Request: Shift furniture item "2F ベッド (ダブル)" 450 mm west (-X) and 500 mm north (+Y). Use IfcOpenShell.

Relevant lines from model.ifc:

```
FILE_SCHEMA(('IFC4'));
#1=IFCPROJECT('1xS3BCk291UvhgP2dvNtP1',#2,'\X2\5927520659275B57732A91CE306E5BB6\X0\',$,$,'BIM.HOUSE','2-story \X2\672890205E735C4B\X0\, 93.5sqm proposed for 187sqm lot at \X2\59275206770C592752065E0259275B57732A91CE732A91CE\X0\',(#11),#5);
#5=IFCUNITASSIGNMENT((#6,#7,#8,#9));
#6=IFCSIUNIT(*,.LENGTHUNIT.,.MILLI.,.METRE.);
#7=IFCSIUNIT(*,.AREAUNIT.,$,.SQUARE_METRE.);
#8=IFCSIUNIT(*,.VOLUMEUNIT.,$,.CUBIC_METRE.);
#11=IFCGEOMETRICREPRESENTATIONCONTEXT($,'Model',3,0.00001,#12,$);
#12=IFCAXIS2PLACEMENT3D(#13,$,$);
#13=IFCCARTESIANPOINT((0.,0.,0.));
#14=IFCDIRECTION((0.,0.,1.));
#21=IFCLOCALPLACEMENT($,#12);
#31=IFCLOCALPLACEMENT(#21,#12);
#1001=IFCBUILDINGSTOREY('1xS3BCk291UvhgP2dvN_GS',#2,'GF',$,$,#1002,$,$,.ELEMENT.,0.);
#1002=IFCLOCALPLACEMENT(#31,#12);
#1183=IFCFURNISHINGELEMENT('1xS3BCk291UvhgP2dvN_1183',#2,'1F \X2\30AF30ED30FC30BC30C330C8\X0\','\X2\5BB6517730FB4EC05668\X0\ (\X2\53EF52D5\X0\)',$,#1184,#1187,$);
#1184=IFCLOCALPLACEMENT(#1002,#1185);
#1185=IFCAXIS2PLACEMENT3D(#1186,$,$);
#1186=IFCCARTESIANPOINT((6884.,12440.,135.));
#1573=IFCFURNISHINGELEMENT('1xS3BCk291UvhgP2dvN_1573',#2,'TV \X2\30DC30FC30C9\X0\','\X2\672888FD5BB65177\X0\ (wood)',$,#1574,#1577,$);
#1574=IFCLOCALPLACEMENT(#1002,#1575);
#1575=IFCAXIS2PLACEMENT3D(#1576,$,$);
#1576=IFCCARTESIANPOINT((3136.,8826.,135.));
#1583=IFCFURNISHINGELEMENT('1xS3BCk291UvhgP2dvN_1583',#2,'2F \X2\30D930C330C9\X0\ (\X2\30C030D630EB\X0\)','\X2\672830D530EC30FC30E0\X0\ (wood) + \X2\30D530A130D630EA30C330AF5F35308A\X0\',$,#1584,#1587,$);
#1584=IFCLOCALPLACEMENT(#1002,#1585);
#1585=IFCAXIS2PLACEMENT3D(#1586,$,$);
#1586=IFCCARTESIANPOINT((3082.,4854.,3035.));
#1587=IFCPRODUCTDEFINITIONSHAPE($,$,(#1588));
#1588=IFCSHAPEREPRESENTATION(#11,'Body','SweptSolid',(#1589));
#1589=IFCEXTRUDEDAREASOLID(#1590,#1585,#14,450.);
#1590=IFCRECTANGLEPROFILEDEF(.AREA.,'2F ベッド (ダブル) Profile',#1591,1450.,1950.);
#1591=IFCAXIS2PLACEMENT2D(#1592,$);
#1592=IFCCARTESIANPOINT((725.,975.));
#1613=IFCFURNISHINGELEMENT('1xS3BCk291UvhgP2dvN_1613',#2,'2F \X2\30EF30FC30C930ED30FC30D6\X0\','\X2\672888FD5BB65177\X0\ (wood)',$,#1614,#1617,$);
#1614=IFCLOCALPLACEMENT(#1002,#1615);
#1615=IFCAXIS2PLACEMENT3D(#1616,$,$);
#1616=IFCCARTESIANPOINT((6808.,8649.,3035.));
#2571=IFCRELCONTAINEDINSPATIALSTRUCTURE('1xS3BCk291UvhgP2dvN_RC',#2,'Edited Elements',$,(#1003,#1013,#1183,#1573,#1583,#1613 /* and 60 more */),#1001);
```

```python
import ifcopenshell
import ifcopenshell.api.geometry
import ifcopenshell.util.placement

model = ifcopenshell.open("model.ifc")

item = model.by_guid("1xS3BCk291UvhgP2dvN_1583")
matrix = ifcopenshell.util.placement.get_local_placement(item.ObjectPlacement)
matrix[0, 3] -= 450.0
matrix[1, 3] += 500.0
ifcopenshell.api.geometry.edit_object_placement(model, product=item, matrix=matrix, is_si=False)

print(ifcopenshell.util.placement.get_local_placement(item.ObjectPlacement).round(3) + 0.0)

model.write("model_edited.ifc")
```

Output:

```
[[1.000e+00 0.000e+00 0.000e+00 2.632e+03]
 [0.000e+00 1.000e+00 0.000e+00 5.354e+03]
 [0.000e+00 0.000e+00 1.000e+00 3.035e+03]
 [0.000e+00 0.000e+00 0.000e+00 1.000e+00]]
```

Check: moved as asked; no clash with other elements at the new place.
